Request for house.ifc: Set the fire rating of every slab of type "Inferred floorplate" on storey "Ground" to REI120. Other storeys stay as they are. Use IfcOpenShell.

First a look at what the model holds.

```python
import ifcopenshell
import ifcopenshell.util.element

model = ifcopenshell.open("house.ifc")
print(model.schema)
storey = next(s for s in model.by_type("IfcBuildingStorey") if s.Name == "Ground")
slabs = [e for e in ifcopenshell.util.element.get_decomposition(storey) if e.is_a("IfcSlab")]
seen = {}
for e in slabs:
    element_type = ifcopenshell.util.element.get_type(e)
    key = (element_type.Name if element_type != e and element_type else None, ifcopenshell.util.element.get_pset(e, "Pset_SlabCommon", "FireRating"))
    seen[key] = seen.get(key, 0) + 1
for (name, value), count in sorted(seen.items(), key=str):
    print(count, "x", name, "|", value)
```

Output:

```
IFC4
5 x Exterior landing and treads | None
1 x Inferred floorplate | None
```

```python
import ifcopenshell
import ifcopenshell.api.pset
import ifcopenshell.util.element

model = ifcopenshell.open("house.ifc")

storey = next(s for s in model.by_type("IfcBuildingStorey") if s.Name == "Ground")
slabs = [e for e in ifcopenshell.util.element.get_decomposition(storey) if e.is_a("IfcSlab")]

count = 0
for e in slabs:
    element_type = ifcopenshell.util.element.get_type(e)
    if element_type in (None, e) or element_type.Name != "Inferred floorplate":
        continue
    # add_pset returns the element's existing set when there is one.
    pset = ifcopenshell.api.pset.add_pset(model, product=e, name="Pset_SlabCommon")
    ifcopenshell.api.pset.edit_pset(model, pset=pset, properties={"FireRating": "REI120"})
    count += 1

print(count, "slabs updated")

model.write("house_updated.ifc")
```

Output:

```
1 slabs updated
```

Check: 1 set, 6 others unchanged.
